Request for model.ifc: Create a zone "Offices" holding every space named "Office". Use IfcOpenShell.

First a look at what the model holds.

```python
import ifcopenshell

model = ifcopenshell.open("model.ifc")
print(model.schema)
seen = {}
for space in model.by_type("IfcSpace"):
    seen[space.LongName] = seen.get(space.LongName, 0) + 1
for name, count in sorted(seen.items(), key=str):
    print(count, "x", name)
print("zones:", [z.Name for z in model.by_type("IfcZone")][:20])
```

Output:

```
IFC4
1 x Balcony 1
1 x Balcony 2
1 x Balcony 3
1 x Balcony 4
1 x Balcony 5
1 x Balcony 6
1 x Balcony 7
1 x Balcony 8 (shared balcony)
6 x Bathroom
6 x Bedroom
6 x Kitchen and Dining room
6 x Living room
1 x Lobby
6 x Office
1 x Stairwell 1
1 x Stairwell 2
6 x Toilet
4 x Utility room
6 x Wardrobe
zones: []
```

```python
import ifcopenshell
import ifcopenshell.api.group
import ifcopenshell.api.root

model = ifcopenshell.open("model.ifc")

names = {"Office"}
spaces = [s for s in model.by_type("IfcSpace") if s.LongName in names]

zone = ifcopenshell.api.root.create_entity(model, ifc_class="IfcZone", name="Offices")
ifcopenshell.api.group.assign_group(model, products=spaces, group=zone)
print(len(spaces), "spaces in", zone.Name)

model.write("model_updated.ifc")
```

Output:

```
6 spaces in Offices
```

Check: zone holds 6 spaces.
